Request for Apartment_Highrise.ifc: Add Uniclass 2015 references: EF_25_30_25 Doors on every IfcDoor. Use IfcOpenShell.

First a look at what the model holds.

```python
import ifcopenshell

model = ifcopenshell.open("Apartment_Highrise.ifc")
print(model.schema)
print("classifications:", [c.Name for c in model.by_type("IfcClassification")])
for ifc_class in ("IfcDoor", "IfcRoof", "IfcStair", "IfcWall", "IfcWindow"):
    print(ifc_class, len(model.by_type(ifc_class)))
```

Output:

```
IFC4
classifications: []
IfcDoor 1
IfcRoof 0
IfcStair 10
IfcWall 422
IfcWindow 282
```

```python
import ifcopenshell
import ifcopenshell.api.classification

model = ifcopenshell.open("Apartment_Highrise.ifc")

system = ifcopenshell.api.classification.add_classification(model, classification="Uniclass 2015")

codes = {
    "IfcDoor": ("EF_25_30_25", "Doors"),
}
for ifc_class, (code, name) in codes.items():
    products = model.by_type(ifc_class)
    ifcopenshell.api.classification.add_reference(
        model, products=products, classification=system, identification=code, name=name
    )
    print(code, len(products))

model.write("Apartment_Highrise_updated.ifc")
```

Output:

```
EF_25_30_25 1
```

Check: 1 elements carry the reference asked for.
